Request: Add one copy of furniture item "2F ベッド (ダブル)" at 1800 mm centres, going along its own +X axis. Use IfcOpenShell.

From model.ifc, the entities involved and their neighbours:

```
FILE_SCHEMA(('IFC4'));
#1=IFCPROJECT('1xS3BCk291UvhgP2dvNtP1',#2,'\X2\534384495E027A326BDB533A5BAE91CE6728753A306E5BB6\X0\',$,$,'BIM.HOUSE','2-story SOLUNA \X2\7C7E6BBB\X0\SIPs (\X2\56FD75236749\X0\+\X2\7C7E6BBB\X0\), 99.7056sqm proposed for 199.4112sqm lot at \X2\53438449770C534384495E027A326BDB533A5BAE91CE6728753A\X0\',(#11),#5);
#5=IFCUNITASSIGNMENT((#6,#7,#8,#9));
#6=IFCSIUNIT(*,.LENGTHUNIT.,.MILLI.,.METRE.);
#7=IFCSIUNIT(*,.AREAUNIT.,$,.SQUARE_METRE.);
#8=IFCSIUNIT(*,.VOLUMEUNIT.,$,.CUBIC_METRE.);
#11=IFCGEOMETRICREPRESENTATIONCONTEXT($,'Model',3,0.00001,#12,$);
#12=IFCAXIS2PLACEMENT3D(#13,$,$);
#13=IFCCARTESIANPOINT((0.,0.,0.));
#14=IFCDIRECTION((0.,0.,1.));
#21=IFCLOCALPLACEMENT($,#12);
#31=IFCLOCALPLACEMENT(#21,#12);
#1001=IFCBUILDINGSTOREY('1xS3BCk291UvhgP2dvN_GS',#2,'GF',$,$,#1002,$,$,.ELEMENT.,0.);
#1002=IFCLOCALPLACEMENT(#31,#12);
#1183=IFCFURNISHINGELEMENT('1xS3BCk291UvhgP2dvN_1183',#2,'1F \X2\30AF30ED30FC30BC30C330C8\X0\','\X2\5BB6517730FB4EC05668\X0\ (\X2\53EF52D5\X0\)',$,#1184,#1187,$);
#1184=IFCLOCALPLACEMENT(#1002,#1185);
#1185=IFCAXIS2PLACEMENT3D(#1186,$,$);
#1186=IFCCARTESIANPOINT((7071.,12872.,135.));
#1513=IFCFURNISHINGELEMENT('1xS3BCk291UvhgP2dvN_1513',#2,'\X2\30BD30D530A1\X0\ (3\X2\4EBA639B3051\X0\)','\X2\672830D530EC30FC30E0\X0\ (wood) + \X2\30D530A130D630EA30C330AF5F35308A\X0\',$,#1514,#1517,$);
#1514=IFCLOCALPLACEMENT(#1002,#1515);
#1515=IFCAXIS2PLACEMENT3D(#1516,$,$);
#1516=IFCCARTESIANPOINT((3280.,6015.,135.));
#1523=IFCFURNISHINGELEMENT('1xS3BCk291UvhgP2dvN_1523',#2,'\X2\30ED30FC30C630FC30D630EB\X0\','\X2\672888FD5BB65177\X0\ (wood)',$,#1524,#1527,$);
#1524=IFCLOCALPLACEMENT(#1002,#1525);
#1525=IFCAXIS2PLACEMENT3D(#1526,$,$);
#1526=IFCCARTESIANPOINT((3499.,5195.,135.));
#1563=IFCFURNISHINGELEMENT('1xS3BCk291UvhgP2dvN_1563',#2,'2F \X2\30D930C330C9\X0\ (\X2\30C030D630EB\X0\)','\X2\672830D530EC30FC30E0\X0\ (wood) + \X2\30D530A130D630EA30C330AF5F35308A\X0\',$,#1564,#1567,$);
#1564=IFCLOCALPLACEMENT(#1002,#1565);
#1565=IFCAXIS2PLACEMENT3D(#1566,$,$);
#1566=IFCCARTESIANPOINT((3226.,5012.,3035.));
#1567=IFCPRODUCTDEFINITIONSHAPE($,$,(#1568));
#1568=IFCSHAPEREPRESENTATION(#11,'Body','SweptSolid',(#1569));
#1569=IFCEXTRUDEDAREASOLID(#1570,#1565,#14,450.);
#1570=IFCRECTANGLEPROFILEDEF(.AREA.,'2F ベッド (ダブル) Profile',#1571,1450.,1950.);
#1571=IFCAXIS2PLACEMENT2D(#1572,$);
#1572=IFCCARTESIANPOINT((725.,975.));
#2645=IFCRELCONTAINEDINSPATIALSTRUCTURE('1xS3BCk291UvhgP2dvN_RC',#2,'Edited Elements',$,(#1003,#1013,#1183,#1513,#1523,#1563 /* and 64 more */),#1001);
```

```python
import ifcopenshell
import ifcopenshell.api.geometry
import ifcopenshell.api.root
import ifcopenshell.util.element
import ifcopenshell.util.placement
import ifcopenshell.util.unit

model = ifcopenshell.open("model.ifc")
unit_scale = ifcopenshell.util.unit.calculate_unit_scale(model)


def reuse_history(source, copy):
    """copy_class also copies each property set's owner history, people and application; keep the originals."""
    for rel in copy.IsDefinedBy:
        if rel.is_a("IfcRelDefinesByProperties") and (history := rel.RelatingPropertyDefinition.OwnerHistory):
            rel.RelatingPropertyDefinition.OwnerHistory = source.OwnerHistory
            ifcopenshell.util.element.remove_deep2(model, history)


source = model.by_id(1563)
base = ifcopenshell.util.placement.get_local_placement(source.ObjectPlacement)
step = base[:3, 0] * 1.8 / unit_scale

for i in range(1, 2):
    copy = ifcopenshell.api.root.copy_class(model, product=source)
    copy.Representation = ifcopenshell.util.element.copy_deep(
        model, source.Representation, exclude=["IfcGeometricRepresentationContext", "IfcRepresentationMap"]
    )
    reuse_history(source, copy)
    matrix = base.copy()
    matrix[:3, 3] += i * step
    print("added at", matrix[:3, 3].round(3) + 0.0)
    ifcopenshell.api.geometry.edit_object_placement(model, product=copy, matrix=matrix, is_si=False)

model.write("model_edited.ifc")
```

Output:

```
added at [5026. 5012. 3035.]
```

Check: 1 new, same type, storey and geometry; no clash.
